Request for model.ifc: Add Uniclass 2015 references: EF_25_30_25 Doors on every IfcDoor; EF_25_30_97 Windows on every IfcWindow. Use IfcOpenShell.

First a look at what the model holds.

```python
import ifcopenshell

model = ifcopenshell.open("model.ifc")
print(model.schema)
print("classifications:", [c.Name for c in model.by_type("IfcClassification")])
for ifc_class in ("IfcDoor", "IfcRoof", "IfcStair", "IfcWall", "IfcWindow"):
    print(ifc_class, len(model.by_type(ifc_class)))
```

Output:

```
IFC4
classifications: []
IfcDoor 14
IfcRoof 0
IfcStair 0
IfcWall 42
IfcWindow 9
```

```python
import ifcopenshell
import ifcopenshell.api.classification

model = ifcopenshell.open("model.ifc")

system = ifcopenshell.api.classification.add_classification(model, classification="Uniclass 2015")

codes = {
    "IfcDoor": ("EF_25_30_25", "Doors"),
    "IfcWindow": ("EF_25_30_97", "Windows"),
}
for ifc_class, (code, name) in codes.items():
    products = model.by_type(ifc_class)
    ifcopenshell.api.classification.add_reference(
        model, products=products, classification=system, identification=code, name=name
    )
    print(code, len(products))

model.write("model_v2.ifc")
```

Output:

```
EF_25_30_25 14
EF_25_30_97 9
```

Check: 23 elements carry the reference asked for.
